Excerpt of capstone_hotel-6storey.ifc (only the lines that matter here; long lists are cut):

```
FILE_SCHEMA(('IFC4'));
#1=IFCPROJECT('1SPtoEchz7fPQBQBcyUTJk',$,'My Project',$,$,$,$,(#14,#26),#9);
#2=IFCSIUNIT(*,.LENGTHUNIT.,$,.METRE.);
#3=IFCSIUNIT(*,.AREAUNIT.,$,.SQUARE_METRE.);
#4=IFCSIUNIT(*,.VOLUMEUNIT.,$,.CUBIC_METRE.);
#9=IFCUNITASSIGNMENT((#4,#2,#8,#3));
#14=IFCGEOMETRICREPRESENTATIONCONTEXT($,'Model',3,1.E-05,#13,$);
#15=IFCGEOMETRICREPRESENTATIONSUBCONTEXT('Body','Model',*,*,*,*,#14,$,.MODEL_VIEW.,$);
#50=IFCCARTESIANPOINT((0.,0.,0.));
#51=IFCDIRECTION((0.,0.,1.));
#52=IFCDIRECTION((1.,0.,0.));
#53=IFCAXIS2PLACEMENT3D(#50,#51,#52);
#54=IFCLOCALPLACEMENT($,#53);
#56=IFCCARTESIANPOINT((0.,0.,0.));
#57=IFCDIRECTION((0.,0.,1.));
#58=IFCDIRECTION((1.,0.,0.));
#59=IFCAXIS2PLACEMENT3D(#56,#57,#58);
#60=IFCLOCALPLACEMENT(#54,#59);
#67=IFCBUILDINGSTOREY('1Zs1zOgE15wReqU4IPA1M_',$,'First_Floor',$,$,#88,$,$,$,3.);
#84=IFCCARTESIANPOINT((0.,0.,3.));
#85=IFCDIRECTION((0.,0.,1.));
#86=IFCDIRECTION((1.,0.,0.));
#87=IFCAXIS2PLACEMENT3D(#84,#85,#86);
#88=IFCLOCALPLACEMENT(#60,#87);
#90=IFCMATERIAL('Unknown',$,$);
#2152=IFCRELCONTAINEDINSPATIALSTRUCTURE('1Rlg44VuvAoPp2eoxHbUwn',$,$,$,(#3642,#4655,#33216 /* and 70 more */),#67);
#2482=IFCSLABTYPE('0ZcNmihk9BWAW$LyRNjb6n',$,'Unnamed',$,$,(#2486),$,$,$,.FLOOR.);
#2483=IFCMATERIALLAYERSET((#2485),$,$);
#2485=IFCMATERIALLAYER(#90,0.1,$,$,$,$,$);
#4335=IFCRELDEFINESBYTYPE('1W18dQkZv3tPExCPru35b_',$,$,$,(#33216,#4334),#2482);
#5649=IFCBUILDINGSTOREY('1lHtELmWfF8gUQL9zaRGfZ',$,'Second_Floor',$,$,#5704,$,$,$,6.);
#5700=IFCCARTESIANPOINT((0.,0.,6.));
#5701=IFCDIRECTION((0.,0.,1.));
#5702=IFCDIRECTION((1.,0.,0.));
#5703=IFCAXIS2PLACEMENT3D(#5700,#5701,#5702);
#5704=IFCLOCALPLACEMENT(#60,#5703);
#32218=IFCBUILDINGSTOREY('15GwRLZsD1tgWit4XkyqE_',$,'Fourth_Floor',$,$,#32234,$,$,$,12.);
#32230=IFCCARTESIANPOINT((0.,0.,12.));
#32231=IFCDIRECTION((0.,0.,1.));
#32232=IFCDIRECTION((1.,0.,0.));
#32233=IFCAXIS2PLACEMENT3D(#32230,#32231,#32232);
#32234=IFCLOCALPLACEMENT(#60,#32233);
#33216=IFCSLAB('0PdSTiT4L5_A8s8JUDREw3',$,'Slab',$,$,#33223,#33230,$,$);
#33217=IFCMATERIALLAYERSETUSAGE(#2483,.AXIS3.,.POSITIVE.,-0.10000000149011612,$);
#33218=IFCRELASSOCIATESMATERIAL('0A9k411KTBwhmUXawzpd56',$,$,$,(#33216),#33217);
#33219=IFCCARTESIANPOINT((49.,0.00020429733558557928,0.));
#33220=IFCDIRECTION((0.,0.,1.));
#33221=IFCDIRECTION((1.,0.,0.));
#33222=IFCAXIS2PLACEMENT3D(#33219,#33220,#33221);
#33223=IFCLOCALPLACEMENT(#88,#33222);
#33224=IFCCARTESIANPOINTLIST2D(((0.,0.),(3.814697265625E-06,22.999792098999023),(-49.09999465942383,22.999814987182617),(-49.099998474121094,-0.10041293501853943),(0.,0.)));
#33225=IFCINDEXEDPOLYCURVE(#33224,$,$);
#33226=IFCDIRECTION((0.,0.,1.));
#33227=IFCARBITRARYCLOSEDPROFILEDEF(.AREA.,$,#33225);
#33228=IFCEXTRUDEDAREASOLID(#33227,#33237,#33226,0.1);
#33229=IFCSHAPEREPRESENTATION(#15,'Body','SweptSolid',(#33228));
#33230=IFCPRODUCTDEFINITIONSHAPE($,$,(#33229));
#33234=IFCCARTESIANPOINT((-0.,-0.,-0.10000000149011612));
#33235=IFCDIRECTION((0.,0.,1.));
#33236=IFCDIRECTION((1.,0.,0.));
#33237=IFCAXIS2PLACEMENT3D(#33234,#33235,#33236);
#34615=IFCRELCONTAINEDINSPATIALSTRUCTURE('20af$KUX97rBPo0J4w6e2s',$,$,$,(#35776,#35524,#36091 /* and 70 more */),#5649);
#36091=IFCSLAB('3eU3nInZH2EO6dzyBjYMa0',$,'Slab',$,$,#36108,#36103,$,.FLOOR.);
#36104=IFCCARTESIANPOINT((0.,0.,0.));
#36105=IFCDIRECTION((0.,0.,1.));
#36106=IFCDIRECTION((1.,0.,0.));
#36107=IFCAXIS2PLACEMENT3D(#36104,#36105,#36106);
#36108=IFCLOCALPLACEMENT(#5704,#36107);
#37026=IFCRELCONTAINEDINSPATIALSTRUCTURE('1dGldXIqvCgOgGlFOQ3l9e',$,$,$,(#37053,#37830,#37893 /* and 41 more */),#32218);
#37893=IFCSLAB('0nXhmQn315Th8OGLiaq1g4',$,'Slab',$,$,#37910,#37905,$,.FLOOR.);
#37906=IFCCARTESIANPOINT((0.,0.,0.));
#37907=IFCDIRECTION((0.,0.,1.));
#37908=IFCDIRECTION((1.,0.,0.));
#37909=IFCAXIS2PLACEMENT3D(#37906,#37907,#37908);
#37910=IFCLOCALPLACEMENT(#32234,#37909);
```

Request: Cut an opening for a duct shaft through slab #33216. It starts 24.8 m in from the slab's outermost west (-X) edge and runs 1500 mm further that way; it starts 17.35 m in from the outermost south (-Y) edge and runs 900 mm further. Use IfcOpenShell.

```python
import numpy as np
import ifcopenshell
import ifcopenshell.api.feature
import ifcopenshell.api.geometry
import ifcopenshell.api.root
import ifcopenshell.geom
import ifcopenshell.util.placement
import ifcopenshell.util.representation
import ifcopenshell.util.shape
import ifcopenshell.util.unit

model = ifcopenshell.open("capstone_hotel-6storey.ifc")
unit_scale = ifcopenshell.util.unit.calculate_unit_scale(model)
settings = ifcopenshell.geom.settings()


def volume(element):
    """Net volume in cubic metres, openings subtracted."""
    shape = ifcopenshell.geom.create_shape(settings, element)
    return ifcopenshell.util.shape.get_volume(shape.geometry)


slab = model.by_id(33216)
before = volume(slab)

# Extent in the slab's own axes, in metres. The edges named are its -X and -Y sides.
slab_shape = ifcopenshell.geom.create_shape(settings, slab)
vertices = ifcopenshell.util.shape.get_vertices(slab_shape.geometry)
x_min, y_min, bottom = vertices.min(axis=0)
top = vertices[:, 2].max()

opening = ifcopenshell.api.root.create_entity(model, ifc_class="IfcOpeningElement", name="Duct shaft opening", predefined_type="OPENING")
context = ifcopenshell.util.representation.get_context(model, "Model", "Body", "MODEL_VIEW")
width, depth = 1.5, 0.9
outline = [(0.0, 0.0), (width, 0.0), (width, depth), (0.0, depth), (0.0, 0.0)]
# Overshoot both faces by 50 mm so the cut is clean.
shape = ifcopenshell.api.geometry.add_slab_representation(
    model, context=context, depth=top - bottom + 0.1, polyline=outline
)
ifcopenshell.api.geometry.assign_representation(model, product=opening, representation=shape)

matrix = ifcopenshell.util.placement.get_local_placement(slab.ObjectPlacement)
matrix[:, 3] = matrix @ np.append(np.array([x_min + 24.8, y_min + 17.35, bottom - 0.05]) / unit_scale, 1.0)
ifcopenshell.api.geometry.edit_object_placement(model, product=opening, matrix=matrix, is_si=False)
ifcopenshell.api.feature.add_feature(model, feature=opening, element=slab)

after = volume(slab)

print(f"slab volume {before:.3f} -> {after:.3f} m3")

model.write("capstone_hotel-6storey_edited.ifc")
```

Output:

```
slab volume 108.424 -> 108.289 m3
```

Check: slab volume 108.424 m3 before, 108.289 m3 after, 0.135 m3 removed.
